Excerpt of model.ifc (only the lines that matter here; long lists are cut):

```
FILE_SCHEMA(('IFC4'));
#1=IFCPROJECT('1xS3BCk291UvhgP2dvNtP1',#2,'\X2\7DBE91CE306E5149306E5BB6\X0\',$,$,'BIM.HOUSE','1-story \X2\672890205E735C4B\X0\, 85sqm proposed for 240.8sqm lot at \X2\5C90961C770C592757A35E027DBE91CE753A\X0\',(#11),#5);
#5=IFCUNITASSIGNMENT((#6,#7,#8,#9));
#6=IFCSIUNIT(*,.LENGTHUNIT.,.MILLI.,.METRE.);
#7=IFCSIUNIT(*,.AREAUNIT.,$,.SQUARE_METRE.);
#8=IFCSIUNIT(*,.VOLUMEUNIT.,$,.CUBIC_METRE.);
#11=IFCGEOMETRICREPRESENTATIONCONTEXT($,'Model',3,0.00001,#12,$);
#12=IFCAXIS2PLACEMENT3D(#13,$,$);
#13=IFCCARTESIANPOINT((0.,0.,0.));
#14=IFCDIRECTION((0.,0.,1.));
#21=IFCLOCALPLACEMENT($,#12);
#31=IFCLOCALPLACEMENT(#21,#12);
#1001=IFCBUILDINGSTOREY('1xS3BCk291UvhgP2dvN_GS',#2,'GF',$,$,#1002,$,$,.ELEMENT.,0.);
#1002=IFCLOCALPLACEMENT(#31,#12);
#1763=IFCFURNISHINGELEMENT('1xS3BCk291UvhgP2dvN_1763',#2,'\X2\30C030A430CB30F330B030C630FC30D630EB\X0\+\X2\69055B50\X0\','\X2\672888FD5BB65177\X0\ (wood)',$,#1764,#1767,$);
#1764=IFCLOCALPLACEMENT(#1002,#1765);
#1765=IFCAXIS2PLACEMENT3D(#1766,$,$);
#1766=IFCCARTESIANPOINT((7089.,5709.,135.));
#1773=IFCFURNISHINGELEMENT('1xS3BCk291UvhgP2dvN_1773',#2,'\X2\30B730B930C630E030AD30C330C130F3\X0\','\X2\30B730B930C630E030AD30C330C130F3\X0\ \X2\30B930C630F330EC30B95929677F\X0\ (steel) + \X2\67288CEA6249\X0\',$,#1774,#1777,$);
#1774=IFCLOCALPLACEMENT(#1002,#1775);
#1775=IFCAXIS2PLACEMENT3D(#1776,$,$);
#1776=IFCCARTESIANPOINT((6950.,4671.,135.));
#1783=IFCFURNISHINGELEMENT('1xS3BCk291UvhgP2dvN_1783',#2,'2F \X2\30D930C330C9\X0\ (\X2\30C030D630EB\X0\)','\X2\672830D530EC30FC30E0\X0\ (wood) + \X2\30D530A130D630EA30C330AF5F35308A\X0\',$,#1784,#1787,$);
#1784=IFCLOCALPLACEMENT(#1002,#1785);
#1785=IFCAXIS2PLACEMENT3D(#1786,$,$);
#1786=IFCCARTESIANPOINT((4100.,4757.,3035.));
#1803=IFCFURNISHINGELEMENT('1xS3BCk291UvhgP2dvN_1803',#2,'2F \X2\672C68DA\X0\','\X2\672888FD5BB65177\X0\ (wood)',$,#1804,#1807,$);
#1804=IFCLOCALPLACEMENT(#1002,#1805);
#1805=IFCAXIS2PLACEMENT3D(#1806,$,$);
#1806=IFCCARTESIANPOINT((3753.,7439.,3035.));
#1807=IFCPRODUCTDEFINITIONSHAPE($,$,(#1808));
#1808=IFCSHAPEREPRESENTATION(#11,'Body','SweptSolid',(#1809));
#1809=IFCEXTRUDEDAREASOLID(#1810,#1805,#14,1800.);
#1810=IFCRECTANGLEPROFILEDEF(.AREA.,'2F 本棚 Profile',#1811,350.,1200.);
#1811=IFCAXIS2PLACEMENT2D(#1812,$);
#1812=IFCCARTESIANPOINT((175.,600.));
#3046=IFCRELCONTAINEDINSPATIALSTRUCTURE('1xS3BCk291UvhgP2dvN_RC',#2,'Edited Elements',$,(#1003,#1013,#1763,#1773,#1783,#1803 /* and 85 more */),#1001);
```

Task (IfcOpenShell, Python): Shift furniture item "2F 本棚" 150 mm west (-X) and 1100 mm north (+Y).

```python
import ifcopenshell
import ifcopenshell.api.geometry
import ifcopenshell.util.placement
import ifcopenshell.util.unit

model = ifcopenshell.open("model.ifc")
unit_scale = ifcopenshell.util.unit.calculate_unit_scale(model)

item = model.by_guid("1xS3BCk291UvhgP2dvN_1803")
matrix = ifcopenshell.util.placement.get_local_placement(item.ObjectPlacement)
matrix[0, 3] -= 0.15 / unit_scale
matrix[1, 3] += 1.1 / unit_scale
ifcopenshell.api.geometry.edit_object_placement(model, product=item, matrix=matrix, is_si=False)

print(ifcopenshell.util.placement.get_local_placement(item.ObjectPlacement).round(3) + 0.0)

model.write("model_rev.ifc")
```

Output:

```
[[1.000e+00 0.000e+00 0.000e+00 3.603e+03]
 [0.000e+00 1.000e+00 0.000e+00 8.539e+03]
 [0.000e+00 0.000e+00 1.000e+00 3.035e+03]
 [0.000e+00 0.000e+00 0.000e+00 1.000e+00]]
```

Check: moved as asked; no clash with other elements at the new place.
